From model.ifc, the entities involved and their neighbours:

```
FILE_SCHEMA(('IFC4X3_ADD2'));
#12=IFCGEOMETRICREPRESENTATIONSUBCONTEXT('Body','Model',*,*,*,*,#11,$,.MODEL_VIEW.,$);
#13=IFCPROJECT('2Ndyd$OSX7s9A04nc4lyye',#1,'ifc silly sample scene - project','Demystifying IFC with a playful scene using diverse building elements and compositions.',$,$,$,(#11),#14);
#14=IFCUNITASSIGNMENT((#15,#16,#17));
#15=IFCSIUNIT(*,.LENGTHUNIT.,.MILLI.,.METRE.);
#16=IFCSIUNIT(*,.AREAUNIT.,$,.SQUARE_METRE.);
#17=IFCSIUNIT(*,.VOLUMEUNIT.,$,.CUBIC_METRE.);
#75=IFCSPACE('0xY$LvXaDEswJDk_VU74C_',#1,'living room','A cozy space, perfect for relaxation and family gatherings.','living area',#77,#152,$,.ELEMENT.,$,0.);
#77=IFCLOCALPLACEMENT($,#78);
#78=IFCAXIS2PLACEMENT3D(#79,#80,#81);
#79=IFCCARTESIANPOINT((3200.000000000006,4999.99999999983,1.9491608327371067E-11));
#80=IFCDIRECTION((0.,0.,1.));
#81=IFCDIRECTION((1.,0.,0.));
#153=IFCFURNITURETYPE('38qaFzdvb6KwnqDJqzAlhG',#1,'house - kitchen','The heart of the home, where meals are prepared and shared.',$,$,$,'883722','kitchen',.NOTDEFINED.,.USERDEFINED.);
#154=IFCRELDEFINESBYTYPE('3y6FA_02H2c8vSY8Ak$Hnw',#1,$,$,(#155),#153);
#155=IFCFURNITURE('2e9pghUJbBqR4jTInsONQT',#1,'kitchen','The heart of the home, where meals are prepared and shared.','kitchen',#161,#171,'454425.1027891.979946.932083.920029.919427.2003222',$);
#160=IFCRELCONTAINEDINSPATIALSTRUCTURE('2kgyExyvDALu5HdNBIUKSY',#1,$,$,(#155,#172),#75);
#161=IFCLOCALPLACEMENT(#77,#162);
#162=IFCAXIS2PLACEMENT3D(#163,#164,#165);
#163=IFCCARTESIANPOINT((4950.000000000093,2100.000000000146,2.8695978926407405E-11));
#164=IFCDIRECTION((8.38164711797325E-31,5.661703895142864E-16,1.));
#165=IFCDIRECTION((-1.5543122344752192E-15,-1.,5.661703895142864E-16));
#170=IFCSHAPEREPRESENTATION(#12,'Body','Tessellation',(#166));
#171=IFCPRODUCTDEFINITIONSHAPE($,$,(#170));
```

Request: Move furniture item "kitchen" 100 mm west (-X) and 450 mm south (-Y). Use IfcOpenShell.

```python
import ifcopenshell
import ifcopenshell.api.geometry
import ifcopenshell.util.placement

model = ifcopenshell.open("model.ifc")

item = model.by_id(155)
matrix = ifcopenshell.util.placement.get_local_placement(item.ObjectPlacement)
matrix[0, 3] -= 100.0
matrix[1, 3] -= 450.0
ifcopenshell.api.geometry.edit_object_placement(model, product=item, matrix=matrix, is_si=False)

print(ifcopenshell.util.placement.get_local_placement(item.ObjectPlacement).round(3) + 0.0)

model.write("model_edited.ifc")
```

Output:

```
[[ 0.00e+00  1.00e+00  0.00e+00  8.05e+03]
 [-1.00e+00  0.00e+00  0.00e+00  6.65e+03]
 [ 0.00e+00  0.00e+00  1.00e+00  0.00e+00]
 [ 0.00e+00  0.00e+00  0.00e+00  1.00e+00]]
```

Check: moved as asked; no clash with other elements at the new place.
